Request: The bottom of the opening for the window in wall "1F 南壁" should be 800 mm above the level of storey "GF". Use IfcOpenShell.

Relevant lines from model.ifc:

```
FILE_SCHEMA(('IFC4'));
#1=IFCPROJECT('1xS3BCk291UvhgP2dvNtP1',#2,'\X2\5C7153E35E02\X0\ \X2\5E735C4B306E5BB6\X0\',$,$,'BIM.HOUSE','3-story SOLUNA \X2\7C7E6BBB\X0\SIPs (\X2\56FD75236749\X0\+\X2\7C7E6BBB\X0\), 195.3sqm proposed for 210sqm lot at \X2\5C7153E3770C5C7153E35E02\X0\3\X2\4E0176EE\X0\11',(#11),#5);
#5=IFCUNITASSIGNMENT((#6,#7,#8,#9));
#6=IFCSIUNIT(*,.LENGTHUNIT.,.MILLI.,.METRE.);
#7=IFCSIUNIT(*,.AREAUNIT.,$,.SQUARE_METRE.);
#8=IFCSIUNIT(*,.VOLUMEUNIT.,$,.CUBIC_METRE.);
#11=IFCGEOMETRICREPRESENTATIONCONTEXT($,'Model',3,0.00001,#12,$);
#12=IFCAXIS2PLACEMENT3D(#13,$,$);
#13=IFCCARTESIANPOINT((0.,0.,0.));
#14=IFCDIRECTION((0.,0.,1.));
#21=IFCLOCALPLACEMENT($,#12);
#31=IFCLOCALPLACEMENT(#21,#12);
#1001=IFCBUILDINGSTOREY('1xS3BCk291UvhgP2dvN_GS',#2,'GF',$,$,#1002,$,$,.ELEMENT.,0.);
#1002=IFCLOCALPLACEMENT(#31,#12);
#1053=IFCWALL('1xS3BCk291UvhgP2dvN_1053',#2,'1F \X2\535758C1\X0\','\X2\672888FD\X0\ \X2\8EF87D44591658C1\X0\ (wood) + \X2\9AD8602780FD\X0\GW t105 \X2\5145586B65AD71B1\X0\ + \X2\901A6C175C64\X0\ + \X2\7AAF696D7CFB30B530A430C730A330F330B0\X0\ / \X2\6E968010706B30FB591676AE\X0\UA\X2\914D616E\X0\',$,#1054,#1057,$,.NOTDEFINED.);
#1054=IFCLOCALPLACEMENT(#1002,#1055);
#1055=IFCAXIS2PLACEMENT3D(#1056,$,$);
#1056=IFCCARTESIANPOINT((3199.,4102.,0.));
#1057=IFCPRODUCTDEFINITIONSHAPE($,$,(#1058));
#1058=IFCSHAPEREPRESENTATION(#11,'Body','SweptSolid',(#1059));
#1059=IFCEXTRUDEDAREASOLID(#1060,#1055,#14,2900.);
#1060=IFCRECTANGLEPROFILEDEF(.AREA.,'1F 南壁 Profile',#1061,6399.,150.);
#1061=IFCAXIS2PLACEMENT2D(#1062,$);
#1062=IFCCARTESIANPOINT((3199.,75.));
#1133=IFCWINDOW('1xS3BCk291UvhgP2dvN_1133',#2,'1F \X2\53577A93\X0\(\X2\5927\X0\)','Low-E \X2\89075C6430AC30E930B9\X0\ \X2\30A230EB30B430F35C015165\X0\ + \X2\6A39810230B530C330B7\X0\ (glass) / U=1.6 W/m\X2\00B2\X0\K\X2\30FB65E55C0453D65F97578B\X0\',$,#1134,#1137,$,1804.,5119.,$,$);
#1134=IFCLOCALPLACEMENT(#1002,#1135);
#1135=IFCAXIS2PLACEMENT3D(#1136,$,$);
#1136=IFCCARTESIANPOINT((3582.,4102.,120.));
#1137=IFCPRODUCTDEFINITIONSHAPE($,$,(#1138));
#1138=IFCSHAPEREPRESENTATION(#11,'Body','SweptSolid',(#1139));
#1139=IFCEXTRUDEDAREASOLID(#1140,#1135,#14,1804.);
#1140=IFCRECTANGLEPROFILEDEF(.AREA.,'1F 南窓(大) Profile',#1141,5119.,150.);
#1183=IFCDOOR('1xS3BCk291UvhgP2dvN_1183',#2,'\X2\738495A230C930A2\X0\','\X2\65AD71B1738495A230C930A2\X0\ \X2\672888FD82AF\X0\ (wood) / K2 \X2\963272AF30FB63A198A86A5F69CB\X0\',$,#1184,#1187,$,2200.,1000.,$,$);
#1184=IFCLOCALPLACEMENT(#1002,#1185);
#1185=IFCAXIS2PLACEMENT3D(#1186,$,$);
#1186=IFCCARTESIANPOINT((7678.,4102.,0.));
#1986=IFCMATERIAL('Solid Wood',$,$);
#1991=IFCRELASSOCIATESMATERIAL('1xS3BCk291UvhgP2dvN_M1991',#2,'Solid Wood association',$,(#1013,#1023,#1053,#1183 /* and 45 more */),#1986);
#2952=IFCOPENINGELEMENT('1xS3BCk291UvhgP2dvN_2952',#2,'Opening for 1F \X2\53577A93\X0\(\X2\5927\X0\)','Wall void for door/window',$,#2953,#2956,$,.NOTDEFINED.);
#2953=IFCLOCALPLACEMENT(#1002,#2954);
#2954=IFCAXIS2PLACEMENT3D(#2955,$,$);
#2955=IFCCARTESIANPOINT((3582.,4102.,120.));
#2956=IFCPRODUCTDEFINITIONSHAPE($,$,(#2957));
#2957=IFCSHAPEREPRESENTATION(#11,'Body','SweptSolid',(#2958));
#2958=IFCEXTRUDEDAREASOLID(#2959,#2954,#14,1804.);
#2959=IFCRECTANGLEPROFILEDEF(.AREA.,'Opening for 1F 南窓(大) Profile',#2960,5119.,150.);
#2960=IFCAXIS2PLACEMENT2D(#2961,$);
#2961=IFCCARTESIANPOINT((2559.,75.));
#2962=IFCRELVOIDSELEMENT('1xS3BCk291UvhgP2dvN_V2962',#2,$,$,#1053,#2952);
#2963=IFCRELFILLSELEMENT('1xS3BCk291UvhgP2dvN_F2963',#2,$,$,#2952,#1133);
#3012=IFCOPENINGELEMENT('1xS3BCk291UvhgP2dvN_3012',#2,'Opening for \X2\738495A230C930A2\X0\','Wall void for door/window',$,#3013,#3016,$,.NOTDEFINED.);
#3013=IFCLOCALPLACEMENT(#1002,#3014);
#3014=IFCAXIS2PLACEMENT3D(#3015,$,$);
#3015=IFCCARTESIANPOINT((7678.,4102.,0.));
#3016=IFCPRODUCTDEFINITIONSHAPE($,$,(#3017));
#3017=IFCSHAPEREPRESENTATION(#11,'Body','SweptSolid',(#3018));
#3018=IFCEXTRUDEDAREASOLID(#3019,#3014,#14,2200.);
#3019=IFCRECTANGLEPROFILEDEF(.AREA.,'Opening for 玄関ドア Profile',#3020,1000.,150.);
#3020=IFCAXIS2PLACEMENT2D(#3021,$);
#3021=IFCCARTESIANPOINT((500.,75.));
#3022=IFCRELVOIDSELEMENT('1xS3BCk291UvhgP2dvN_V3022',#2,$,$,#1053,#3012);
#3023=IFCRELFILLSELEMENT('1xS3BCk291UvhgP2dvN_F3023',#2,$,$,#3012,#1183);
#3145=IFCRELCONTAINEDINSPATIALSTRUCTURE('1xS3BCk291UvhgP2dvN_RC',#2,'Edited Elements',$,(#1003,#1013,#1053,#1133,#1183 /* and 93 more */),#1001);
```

```python
import numpy as np
import ifcopenshell
import ifcopenshell.api.geometry
import ifcopenshell.geom
import ifcopenshell.util.element
import ifcopenshell.util.placement
import ifcopenshell.util.shape
import ifcopenshell.util.unit

model = ifcopenshell.open("model.ifc")
unit_scale = ifcopenshell.util.unit.calculate_unit_scale(model)

window = model.by_guid("1xS3BCk291UvhgP2dvN_1133")
opening = window.FillsVoids[0].RelatingOpeningElement
storey = ifcopenshell.util.element.get_container(window, ifc_class="IfcBuildingStorey")
level = ifcopenshell.util.placement.get_local_placement(storey.ObjectPlacement)[2, 3]

# The opening's origin need not be at the sill, so measure its lowest point.
shape = ifcopenshell.geom.create_shape(ifcopenshell.geom.settings(), opening)
bottom = ifcopenshell.util.shape.get_shape_bottom_elevation(shape, shape.geometry) / unit_scale
dz = level + 0.8 / unit_scale - bottom

shift = np.array([0.0, 0.0, dz])
# The window is not placed relative to its opening, so move both.
for product in (opening, window):
    matrix = ifcopenshell.util.placement.get_local_placement(product.ObjectPlacement)
    matrix[:3, 3] += shift
    ifcopenshell.api.geometry.edit_object_placement(model, product=product, matrix=matrix, is_si=False)

print(f"moved by {dz * unit_scale:+.3f} m")

model.write("model_rev.ifc")
```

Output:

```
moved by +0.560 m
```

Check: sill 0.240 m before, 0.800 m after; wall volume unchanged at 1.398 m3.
